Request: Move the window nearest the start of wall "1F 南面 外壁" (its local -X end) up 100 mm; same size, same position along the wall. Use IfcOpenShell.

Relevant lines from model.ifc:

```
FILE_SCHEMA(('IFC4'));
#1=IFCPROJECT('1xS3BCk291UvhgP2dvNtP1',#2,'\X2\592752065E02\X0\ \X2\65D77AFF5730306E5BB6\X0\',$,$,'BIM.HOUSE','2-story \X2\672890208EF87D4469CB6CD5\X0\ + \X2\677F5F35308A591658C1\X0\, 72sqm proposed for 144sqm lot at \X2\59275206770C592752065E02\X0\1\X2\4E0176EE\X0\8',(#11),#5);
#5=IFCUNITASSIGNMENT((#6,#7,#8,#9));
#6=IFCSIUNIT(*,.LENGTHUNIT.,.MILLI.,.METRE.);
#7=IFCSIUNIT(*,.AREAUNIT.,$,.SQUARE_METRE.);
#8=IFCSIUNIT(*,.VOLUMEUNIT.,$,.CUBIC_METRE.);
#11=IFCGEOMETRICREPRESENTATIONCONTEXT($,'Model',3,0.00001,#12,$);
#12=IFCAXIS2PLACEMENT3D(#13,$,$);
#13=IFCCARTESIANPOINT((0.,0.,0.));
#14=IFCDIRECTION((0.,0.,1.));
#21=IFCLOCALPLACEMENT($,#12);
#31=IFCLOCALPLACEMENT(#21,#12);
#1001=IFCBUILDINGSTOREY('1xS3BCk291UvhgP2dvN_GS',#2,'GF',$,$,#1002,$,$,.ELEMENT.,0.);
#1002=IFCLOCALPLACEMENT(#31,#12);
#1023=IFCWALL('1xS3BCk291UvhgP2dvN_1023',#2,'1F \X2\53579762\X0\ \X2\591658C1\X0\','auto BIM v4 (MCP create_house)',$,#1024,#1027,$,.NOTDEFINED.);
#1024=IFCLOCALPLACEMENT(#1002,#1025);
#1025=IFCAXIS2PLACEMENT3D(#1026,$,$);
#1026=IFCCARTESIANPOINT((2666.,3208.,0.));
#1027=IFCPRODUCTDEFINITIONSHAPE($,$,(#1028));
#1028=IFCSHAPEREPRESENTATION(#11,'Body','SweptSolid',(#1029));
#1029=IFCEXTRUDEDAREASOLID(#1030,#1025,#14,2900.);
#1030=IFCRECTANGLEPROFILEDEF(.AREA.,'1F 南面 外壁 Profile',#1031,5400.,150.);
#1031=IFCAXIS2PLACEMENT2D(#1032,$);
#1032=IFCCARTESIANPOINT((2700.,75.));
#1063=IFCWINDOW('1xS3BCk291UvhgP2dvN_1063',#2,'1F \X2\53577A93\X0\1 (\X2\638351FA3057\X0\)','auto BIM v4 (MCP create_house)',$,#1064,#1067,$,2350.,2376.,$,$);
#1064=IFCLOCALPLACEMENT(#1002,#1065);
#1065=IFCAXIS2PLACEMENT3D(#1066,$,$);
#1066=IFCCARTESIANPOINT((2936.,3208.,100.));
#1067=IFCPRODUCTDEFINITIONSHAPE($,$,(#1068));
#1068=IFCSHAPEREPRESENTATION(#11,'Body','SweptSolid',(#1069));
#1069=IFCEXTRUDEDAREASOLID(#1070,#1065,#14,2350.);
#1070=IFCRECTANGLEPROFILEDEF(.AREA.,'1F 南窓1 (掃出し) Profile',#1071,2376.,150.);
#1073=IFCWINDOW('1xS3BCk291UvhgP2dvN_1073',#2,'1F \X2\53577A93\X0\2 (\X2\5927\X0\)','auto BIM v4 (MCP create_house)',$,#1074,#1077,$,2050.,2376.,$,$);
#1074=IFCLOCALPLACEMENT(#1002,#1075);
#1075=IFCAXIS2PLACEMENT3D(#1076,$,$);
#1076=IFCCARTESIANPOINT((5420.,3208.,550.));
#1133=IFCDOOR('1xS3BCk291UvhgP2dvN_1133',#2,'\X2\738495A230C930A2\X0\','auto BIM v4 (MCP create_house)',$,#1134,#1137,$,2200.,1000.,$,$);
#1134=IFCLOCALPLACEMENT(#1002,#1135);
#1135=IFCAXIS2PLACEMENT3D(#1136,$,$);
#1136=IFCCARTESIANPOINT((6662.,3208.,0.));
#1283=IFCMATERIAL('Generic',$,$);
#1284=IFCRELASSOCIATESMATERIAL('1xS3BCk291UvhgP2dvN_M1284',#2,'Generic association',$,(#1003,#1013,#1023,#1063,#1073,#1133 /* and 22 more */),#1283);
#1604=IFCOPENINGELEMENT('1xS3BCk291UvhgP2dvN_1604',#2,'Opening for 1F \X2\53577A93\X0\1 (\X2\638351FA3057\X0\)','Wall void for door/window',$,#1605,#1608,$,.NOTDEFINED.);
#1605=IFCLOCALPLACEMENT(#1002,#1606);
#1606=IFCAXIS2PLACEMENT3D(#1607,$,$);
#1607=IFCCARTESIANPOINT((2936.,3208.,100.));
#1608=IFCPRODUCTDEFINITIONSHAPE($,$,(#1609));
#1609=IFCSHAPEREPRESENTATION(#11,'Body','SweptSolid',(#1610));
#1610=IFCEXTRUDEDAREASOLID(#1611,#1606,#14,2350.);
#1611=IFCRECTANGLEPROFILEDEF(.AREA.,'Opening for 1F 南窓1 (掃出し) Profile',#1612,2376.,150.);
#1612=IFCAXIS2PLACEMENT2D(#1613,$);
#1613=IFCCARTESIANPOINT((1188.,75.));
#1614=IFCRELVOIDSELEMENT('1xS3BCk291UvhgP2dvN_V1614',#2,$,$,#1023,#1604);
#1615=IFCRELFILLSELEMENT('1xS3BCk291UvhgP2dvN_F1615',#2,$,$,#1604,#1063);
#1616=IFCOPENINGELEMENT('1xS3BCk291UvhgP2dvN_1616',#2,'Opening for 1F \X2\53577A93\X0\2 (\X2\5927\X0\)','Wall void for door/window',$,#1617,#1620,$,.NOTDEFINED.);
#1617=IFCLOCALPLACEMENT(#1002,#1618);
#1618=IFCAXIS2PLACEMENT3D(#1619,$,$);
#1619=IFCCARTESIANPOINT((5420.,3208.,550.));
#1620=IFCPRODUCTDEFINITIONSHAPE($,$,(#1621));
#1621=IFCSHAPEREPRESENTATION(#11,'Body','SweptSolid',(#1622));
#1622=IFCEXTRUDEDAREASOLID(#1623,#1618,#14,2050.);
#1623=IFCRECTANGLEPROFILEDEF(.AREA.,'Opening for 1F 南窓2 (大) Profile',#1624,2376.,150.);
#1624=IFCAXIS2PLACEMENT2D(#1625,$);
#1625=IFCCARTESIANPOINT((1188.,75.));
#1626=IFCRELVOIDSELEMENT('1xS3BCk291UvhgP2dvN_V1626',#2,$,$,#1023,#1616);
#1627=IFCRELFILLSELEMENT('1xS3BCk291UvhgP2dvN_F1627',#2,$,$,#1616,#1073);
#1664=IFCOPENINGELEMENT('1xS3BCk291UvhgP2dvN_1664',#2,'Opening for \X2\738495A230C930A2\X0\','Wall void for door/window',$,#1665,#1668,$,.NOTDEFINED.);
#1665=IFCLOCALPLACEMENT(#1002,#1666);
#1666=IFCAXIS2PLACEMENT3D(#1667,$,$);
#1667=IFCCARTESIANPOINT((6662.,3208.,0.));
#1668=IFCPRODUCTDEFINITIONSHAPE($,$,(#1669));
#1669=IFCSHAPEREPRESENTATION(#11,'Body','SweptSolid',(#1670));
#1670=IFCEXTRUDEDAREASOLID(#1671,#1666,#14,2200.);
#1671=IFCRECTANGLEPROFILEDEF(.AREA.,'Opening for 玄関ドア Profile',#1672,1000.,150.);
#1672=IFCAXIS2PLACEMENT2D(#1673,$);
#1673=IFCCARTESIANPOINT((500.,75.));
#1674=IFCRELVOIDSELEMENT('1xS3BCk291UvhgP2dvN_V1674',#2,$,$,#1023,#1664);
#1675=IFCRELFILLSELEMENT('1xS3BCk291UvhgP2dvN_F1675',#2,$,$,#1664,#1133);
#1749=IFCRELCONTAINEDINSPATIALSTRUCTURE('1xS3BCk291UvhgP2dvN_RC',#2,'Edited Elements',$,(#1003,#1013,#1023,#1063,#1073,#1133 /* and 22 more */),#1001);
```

```python
import numpy as np
import ifcopenshell
import ifcopenshell.api.geometry
import ifcopenshell.util.placement
import ifcopenshell.util.unit

model = ifcopenshell.open("model.ifc")
unit_scale = ifcopenshell.util.unit.calculate_unit_scale(model)

window = model.by_guid("1xS3BCk291UvhgP2dvN_1063")
opening = window.FillsVoids[0].RelatingOpeningElement
dz = 100.0

shift = np.array([0.0, 0.0, dz])
# The window is not placed relative to its opening, so move both.
for product in (opening, window):
    matrix = ifcopenshell.util.placement.get_local_placement(product.ObjectPlacement)
    matrix[:3, 3] += shift
    ifcopenshell.api.geometry.edit_object_placement(model, product=product, matrix=matrix, is_si=False)

print(f"moved by {dz * unit_scale:+.3f} m")

model.write("model_rev.ifc")
```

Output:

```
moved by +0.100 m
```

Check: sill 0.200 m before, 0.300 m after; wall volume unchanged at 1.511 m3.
